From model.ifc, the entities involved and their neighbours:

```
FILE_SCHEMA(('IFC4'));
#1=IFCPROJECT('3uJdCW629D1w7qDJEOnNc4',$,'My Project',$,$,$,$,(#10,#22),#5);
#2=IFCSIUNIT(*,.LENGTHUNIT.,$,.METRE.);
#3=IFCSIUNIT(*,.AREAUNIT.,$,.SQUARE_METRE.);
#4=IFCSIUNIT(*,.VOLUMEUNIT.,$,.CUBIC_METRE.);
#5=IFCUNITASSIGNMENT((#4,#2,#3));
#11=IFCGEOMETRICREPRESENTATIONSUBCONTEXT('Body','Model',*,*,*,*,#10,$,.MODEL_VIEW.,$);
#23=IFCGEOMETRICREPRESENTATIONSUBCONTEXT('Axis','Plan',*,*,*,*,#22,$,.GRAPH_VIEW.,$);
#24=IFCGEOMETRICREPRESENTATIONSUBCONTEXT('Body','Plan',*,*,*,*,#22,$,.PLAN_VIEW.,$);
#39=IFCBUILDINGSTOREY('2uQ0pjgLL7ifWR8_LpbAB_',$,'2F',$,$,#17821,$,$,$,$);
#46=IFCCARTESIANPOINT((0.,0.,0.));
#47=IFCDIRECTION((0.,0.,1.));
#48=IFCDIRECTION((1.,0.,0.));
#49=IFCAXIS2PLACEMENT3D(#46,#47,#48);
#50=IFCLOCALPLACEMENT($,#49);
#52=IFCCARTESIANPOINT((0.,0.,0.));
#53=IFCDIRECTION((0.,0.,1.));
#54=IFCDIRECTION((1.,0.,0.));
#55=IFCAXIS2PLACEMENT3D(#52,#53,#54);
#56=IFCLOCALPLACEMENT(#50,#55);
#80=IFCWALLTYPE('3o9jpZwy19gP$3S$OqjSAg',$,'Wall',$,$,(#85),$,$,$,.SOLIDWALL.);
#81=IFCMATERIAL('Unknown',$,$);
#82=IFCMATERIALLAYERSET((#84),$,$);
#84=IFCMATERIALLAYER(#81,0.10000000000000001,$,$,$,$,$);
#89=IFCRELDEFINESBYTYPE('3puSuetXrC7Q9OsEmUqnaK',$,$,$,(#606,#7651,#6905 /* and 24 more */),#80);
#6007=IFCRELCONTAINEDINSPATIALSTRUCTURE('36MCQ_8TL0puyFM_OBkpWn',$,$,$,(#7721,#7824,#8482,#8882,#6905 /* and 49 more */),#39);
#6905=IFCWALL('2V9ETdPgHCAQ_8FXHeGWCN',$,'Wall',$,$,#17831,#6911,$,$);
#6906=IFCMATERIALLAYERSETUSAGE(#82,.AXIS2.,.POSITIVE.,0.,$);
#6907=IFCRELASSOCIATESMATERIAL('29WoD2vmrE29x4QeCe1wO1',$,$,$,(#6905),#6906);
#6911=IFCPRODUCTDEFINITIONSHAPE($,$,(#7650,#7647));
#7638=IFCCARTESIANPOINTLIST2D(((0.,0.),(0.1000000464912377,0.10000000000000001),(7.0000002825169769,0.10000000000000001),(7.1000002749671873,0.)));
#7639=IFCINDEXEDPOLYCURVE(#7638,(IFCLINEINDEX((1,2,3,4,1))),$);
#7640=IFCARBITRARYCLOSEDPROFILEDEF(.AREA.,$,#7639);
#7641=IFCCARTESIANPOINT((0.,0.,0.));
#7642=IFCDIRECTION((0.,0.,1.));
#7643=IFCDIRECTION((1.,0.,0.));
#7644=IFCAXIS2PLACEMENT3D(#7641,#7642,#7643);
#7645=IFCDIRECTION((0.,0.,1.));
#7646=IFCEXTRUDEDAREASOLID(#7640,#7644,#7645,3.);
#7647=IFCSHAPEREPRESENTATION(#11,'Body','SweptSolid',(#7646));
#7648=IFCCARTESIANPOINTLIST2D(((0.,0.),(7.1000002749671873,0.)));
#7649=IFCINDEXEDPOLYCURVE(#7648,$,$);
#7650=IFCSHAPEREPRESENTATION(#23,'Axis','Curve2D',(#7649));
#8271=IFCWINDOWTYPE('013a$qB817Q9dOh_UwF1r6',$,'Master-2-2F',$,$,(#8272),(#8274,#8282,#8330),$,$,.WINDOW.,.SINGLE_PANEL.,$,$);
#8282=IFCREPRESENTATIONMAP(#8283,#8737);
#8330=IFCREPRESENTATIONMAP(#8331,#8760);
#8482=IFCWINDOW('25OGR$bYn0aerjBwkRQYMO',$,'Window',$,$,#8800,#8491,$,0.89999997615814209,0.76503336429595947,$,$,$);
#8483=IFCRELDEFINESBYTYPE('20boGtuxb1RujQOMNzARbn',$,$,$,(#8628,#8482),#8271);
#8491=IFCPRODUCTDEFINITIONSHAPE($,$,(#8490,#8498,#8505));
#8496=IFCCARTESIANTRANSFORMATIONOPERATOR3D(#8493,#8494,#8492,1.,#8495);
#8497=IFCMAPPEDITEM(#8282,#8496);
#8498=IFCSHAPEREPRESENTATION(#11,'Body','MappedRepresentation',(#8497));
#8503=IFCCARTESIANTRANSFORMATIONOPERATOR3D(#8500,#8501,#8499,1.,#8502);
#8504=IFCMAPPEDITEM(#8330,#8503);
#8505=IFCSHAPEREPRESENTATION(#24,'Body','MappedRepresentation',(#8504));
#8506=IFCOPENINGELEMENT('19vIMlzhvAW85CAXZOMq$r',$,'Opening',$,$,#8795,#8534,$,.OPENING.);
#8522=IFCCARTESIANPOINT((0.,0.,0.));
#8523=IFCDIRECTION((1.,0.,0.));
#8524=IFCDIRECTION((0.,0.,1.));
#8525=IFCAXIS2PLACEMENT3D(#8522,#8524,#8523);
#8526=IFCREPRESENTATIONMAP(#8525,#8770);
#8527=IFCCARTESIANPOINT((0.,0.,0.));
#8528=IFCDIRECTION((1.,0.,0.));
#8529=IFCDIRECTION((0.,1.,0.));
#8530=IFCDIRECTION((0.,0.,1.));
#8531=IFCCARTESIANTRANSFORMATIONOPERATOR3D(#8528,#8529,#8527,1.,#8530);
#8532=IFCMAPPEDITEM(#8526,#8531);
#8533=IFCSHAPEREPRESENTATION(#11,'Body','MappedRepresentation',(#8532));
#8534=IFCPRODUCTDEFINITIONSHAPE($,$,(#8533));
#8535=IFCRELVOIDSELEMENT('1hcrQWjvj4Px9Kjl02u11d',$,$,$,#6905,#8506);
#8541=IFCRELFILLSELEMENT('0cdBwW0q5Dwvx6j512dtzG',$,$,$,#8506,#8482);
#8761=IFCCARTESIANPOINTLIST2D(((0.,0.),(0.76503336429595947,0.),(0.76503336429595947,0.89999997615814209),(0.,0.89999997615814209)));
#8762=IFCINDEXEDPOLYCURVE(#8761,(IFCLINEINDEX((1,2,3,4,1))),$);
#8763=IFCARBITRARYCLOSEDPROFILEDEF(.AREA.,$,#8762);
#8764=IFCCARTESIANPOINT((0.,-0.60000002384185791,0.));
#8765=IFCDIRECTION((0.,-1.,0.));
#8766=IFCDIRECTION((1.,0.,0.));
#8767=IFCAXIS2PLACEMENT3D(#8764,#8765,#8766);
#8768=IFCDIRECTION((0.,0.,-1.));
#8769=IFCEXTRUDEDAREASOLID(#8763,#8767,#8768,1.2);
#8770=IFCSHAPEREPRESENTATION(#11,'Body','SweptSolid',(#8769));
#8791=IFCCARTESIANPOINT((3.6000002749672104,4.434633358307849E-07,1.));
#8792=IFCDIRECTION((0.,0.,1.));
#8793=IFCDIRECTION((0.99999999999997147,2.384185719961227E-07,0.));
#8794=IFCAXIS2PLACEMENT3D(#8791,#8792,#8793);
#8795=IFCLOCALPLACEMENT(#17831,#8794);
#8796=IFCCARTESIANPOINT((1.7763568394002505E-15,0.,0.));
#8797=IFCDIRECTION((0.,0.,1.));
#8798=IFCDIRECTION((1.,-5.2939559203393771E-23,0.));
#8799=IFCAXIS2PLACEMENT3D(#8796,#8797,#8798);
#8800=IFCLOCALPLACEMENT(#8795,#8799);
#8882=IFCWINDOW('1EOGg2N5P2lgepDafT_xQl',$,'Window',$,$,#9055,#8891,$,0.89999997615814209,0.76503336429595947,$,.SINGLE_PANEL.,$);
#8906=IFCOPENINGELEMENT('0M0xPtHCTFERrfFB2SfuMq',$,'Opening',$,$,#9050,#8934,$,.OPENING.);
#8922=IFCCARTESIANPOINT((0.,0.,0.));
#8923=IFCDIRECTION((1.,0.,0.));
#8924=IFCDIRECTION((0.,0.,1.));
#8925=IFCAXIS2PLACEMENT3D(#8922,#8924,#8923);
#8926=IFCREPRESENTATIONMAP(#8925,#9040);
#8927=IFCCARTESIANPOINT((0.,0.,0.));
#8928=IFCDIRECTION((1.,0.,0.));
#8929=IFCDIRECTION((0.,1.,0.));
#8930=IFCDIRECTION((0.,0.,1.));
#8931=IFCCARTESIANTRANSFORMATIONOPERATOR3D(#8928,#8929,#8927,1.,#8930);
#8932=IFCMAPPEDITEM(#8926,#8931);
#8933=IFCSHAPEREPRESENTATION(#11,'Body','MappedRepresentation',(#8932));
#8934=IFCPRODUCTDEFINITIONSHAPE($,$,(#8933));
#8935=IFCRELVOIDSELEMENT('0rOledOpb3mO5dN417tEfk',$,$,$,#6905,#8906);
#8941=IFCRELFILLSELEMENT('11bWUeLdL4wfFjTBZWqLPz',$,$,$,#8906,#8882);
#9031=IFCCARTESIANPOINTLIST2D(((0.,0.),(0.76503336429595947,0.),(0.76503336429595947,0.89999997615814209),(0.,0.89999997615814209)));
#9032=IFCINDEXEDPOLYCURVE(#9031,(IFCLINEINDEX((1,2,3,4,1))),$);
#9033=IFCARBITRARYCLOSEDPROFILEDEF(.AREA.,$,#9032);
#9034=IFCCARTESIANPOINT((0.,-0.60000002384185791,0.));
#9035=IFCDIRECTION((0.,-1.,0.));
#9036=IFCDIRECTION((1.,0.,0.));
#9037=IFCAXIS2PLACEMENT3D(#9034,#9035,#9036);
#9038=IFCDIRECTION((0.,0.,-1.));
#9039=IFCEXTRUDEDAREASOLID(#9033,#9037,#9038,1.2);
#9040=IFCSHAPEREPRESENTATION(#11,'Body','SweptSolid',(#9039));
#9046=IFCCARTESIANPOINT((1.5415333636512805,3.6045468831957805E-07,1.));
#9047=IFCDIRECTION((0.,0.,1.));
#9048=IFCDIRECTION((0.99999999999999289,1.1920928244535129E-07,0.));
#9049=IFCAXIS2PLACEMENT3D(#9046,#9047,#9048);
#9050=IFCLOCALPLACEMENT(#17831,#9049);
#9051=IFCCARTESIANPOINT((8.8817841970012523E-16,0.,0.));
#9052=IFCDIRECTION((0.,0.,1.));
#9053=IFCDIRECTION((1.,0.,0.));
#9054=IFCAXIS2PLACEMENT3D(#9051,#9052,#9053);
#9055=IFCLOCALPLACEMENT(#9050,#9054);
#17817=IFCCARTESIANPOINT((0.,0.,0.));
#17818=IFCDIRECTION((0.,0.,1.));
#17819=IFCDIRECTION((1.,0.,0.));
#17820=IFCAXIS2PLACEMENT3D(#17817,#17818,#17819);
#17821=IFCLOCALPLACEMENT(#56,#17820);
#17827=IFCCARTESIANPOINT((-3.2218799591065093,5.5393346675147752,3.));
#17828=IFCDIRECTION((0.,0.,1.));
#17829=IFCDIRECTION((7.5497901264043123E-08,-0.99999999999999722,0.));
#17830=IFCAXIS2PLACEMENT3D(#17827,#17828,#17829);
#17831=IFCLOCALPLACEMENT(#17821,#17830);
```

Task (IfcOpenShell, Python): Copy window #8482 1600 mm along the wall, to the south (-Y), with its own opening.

```python
import ifcopenshell
import ifcopenshell.api.feature
import ifcopenshell.api.geometry
import ifcopenshell.api.root
import ifcopenshell.geom
import ifcopenshell.util.element
import ifcopenshell.util.placement
import ifcopenshell.util.shape

model = ifcopenshell.open("model.ifc")
settings = ifcopenshell.geom.settings()


def volume(element):
    """Net volume in cubic metres, openings subtracted."""
    shape = ifcopenshell.geom.create_shape(settings, element)
    return ifcopenshell.util.shape.get_volume(shape.geometry)


window = model.by_id(8482)
opening = window.FillsVoids[0].RelatingOpeningElement
wall = opening.VoidsElements[0].RelatingBuildingElement
before = volume(wall)
shift = ifcopenshell.util.placement.get_local_placement(wall.ObjectPlacement)[:3, 0] * 1.6

# copy_class copies the void relationship, type, container and properties, but no geometry.
new_opening = ifcopenshell.api.root.copy_class(model, product=opening)
new_opening.Representation = ifcopenshell.util.element.copy_deep(
    model, opening.Representation, exclude=["IfcGeometricRepresentationContext", "IfcRepresentationMap"]
)
new_window = ifcopenshell.api.root.copy_class(model, product=window)
new_window.Representation = ifcopenshell.util.element.copy_deep(
    model, window.Representation, exclude=["IfcGeometricRepresentationContext", "IfcRepresentationMap"]
)
ifcopenshell.api.feature.add_filling(model, opening=new_opening, element=new_window)

for old, new in ((opening, new_opening), (window, new_window)):
    matrix = ifcopenshell.util.placement.get_local_placement(old.ObjectPlacement)
    matrix[:3, 3] += shift
    ifcopenshell.api.geometry.edit_object_placement(model, product=new, matrix=matrix, is_si=False)

after = volume(wall)

print(f"wall volume {before:.3f} -> {after:.3f} m3")

model.write("model_v2.ifc")
```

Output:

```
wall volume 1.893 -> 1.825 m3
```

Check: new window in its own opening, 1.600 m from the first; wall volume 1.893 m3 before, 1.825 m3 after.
